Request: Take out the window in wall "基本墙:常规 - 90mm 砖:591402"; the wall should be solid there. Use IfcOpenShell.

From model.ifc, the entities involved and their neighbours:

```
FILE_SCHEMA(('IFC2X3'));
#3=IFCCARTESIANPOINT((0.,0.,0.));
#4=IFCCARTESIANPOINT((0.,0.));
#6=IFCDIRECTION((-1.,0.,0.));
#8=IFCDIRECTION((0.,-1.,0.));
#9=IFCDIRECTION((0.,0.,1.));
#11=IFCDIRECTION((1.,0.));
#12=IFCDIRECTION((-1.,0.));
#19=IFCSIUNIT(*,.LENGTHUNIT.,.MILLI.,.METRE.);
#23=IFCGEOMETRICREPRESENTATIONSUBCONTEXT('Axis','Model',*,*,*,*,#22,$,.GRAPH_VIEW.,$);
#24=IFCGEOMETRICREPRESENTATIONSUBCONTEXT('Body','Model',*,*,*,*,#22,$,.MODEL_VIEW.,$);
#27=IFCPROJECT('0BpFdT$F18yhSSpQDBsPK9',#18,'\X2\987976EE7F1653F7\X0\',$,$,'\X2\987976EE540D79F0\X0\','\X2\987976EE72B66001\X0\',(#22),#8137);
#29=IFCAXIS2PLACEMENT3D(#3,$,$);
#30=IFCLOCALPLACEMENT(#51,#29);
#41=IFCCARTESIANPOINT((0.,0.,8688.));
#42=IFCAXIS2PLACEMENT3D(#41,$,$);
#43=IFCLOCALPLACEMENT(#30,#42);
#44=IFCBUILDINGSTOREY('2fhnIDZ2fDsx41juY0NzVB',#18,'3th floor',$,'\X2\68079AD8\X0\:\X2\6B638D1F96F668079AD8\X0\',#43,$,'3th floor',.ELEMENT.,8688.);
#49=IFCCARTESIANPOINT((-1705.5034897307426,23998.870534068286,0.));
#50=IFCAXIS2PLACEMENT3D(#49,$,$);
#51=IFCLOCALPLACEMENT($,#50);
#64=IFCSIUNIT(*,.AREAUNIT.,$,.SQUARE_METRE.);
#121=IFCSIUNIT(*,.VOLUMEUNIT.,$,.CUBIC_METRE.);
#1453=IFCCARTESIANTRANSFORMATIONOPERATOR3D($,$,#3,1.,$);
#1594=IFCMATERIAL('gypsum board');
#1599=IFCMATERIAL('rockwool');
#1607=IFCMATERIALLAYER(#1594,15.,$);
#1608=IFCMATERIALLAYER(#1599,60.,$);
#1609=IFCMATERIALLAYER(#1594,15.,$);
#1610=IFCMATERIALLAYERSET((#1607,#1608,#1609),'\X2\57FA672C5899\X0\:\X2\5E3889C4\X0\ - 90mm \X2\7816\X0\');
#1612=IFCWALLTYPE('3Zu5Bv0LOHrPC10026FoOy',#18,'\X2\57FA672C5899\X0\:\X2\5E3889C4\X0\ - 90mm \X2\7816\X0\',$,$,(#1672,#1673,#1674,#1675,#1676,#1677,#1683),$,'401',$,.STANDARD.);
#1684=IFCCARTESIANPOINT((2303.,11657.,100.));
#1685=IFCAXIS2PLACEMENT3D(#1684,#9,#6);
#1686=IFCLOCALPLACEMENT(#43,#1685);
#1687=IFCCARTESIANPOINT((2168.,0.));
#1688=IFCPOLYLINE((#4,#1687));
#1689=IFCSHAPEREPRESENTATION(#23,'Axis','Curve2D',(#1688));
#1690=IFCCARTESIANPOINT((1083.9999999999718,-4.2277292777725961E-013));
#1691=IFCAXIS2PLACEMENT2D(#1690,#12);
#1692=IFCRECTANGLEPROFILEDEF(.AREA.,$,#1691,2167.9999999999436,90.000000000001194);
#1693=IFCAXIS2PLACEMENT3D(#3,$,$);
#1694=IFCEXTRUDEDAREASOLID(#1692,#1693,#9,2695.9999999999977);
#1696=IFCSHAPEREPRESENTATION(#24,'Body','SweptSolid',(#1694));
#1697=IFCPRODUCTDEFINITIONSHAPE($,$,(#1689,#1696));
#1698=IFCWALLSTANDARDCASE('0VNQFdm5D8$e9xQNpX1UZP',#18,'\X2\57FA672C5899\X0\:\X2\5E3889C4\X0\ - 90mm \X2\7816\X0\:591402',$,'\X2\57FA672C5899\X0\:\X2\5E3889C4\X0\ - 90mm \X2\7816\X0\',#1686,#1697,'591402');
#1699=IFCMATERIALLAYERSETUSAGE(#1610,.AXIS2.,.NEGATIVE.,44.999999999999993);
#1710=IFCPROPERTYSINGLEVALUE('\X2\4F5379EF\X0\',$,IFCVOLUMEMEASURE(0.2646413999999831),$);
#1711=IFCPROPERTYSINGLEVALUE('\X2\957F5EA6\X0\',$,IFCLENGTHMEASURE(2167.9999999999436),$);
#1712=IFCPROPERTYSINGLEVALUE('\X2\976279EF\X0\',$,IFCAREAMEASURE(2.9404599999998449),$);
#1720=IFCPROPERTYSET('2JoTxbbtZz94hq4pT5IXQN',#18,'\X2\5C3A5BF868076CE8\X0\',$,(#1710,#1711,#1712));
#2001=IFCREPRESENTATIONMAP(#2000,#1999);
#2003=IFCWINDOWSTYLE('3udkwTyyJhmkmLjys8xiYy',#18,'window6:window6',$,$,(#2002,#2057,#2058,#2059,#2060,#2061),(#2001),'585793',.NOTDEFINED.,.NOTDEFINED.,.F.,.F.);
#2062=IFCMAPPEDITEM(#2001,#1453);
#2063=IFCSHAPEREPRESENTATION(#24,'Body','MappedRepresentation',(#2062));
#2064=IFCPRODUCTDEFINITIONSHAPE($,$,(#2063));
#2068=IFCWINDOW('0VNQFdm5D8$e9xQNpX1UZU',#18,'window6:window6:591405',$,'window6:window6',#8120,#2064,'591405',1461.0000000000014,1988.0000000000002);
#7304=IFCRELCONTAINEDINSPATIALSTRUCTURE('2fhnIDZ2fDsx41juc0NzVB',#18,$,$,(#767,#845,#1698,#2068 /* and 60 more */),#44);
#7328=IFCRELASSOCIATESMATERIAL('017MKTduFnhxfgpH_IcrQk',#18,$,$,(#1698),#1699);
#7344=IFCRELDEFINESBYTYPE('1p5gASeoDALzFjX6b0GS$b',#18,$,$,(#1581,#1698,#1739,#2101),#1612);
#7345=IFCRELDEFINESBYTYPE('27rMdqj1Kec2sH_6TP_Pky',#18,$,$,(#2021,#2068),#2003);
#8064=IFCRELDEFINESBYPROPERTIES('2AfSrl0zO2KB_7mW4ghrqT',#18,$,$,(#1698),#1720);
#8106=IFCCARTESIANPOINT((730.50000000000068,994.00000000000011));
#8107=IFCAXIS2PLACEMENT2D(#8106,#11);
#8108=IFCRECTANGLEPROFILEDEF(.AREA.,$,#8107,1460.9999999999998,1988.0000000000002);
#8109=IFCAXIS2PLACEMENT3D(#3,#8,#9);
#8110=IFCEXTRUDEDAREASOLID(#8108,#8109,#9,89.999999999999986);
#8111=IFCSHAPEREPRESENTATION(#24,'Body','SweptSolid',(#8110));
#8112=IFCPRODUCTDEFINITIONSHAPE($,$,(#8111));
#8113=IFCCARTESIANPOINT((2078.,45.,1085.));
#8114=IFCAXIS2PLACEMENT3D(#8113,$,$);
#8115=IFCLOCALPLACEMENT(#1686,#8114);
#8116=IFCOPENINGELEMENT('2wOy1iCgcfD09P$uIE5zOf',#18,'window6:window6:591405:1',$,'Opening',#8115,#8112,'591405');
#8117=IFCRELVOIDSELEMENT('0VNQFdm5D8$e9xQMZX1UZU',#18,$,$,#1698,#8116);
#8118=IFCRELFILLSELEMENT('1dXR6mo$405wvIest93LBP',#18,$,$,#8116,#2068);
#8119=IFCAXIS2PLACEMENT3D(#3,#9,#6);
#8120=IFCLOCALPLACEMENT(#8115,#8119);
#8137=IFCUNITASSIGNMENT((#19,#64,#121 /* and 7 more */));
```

```python
import ifcopenshell
import ifcopenshell.api.feature
import ifcopenshell.api.pset
import ifcopenshell.api.root
import ifcopenshell.geom
import ifcopenshell.util.element
import ifcopenshell.util.shape
import ifcopenshell.util.unit

model = ifcopenshell.open("model.ifc")
area_scale = ifcopenshell.util.unit.calculate_unit_scale(model, "AREAUNIT")
volume_scale = ifcopenshell.util.unit.calculate_unit_scale(model, "VOLUMEUNIT")
settings = ifcopenshell.geom.settings()


def volume(element):
    """Net volume in cubic metres, openings subtracted."""
    shape = ifcopenshell.geom.create_shape(settings, element)
    return ifcopenshell.util.shape.get_volume(shape.geometry)


window = model.by_guid("0VNQFdm5D8$e9xQNpX1UZU")
opening = window.FillsVoids[0].RelatingOpeningElement
wall = opening.VoidsElements[0].RelatingBuildingElement
before = volume(wall)

ifcopenshell.api.root.remove_product(model, product=window)
ifcopenshell.api.feature.remove_feature(model, feature=opening)

after = volume(wall)
thickness = 0.09  # wall thickness in metres

# Update the wall's stored quantities.
pset = model.by_id(ifcopenshell.util.element.get_pset(wall, "尺寸标注", should_inherit=False)["id"])
ifcopenshell.api.pset.edit_pset(model, pset=pset, properties={
    "体积": model.create_entity("IfcVolumeMeasure", after / volume_scale),
    "面积": model.create_entity("IfcAreaMeasure", after / thickness / area_scale),
})

print(f"wall volume {before:.3f} -> {after:.3f} m3")

model.write("model-out.ifc")
```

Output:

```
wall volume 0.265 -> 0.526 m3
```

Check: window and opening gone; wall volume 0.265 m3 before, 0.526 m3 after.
